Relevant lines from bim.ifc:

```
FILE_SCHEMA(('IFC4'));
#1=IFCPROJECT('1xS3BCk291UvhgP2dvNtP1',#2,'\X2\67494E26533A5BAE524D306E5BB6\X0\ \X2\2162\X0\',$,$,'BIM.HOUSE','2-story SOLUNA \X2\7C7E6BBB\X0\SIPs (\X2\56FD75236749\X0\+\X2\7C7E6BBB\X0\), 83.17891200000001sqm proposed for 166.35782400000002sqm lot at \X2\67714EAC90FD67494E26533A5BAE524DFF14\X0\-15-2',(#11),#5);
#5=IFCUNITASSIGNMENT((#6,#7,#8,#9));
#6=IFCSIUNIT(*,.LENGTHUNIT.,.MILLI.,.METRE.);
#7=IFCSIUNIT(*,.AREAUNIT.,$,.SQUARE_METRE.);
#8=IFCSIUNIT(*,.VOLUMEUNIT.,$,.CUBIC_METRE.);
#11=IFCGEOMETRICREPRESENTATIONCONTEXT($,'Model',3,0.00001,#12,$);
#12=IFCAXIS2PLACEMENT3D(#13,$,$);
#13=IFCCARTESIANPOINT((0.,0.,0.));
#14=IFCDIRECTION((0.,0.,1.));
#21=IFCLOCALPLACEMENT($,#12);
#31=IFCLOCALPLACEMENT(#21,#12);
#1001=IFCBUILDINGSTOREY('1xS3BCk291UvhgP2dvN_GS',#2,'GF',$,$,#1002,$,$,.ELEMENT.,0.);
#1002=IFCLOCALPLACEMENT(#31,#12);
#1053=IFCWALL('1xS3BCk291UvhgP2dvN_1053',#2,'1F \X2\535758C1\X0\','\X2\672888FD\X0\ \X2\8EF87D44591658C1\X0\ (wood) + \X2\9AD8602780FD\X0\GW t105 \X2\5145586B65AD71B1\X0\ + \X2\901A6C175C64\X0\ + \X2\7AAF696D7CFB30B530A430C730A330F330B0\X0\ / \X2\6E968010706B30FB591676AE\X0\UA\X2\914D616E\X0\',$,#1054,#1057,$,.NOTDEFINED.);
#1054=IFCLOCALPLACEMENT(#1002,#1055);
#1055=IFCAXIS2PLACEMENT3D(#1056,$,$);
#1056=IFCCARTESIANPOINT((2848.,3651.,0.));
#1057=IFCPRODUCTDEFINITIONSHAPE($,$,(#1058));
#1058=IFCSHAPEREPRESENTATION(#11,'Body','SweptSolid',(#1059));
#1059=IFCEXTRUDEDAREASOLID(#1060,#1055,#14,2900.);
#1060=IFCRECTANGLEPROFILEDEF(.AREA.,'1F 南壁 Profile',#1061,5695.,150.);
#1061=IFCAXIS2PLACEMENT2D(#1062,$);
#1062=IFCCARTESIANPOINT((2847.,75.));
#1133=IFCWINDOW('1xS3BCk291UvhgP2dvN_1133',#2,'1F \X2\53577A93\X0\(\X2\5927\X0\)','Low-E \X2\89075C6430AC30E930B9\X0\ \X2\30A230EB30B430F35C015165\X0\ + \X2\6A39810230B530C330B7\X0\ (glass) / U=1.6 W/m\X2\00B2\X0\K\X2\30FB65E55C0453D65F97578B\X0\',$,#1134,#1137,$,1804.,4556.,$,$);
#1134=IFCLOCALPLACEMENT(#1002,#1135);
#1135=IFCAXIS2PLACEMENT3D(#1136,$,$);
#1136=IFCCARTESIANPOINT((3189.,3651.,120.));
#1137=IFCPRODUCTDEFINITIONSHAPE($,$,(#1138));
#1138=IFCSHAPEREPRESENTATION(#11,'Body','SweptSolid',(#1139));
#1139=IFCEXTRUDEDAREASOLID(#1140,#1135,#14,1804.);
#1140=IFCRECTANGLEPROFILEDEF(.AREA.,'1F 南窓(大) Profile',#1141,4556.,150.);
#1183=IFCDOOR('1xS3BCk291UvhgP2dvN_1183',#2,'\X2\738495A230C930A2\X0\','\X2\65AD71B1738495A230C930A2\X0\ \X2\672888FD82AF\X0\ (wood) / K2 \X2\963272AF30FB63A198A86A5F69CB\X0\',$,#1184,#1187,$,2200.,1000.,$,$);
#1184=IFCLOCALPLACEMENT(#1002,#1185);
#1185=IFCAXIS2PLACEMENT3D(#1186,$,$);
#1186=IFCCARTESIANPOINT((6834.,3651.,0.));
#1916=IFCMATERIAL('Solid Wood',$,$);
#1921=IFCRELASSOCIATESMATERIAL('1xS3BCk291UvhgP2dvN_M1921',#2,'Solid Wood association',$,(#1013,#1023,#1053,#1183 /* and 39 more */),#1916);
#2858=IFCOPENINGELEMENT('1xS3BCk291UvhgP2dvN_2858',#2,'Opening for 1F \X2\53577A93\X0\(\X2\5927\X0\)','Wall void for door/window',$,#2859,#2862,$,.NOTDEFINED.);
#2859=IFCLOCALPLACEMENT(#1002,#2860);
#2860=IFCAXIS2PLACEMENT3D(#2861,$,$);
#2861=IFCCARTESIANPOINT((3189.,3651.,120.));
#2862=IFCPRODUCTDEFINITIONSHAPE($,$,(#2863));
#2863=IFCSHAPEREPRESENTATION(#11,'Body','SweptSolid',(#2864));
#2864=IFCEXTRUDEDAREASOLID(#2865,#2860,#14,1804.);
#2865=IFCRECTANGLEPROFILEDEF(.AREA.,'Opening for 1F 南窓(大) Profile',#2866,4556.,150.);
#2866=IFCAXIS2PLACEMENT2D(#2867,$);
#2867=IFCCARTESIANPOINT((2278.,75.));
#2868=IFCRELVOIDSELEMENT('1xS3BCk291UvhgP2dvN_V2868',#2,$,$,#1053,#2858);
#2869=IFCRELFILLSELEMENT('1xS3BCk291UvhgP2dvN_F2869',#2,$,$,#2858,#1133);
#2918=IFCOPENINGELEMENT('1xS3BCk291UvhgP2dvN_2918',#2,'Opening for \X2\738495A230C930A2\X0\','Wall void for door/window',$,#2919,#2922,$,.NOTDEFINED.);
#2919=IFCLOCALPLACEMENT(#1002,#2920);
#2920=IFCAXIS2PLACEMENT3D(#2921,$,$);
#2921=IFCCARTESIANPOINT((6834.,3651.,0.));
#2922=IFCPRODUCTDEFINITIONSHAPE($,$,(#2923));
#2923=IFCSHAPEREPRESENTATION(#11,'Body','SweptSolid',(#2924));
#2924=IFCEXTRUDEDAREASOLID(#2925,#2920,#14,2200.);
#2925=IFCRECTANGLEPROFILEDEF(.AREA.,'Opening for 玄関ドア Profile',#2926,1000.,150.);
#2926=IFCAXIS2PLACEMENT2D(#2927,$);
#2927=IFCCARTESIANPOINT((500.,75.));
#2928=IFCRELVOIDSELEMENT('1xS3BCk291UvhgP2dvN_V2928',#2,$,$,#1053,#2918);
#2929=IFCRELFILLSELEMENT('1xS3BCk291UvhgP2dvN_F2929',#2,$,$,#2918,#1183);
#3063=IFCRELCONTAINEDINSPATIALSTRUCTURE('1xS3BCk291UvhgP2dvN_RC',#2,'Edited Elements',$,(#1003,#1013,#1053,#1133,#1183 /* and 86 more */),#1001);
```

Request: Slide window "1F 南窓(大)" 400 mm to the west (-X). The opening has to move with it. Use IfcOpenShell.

```python
import ifcopenshell
import ifcopenshell.api.geometry
import ifcopenshell.util.placement
import ifcopenshell.util.unit

model = ifcopenshell.open("bim.ifc")
unit_scale = ifcopenshell.util.unit.calculate_unit_scale(model)

window = model.by_guid("1xS3BCk291UvhgP2dvN_1133")
opening = window.FillsVoids[0].RelatingOpeningElement
wall = opening.VoidsElements[0].RelatingBuildingElement

wall_matrix = ifcopenshell.util.placement.get_local_placement(wall.ObjectPlacement)
shift = wall_matrix[:3, 0] * -0.4 / unit_scale
before = ifcopenshell.util.placement.get_local_placement(window.ObjectPlacement)[:3, 3].copy()

# The window is not placed relative to its opening, so move both.
for product in (opening, window):
    matrix = ifcopenshell.util.placement.get_local_placement(product.ObjectPlacement)
    matrix[:3, 3] += shift
    ifcopenshell.api.geometry.edit_object_placement(model, product=product, matrix=matrix, is_si=False)

after = ifcopenshell.util.placement.get_local_placement(window.ObjectPlacement)[:3, 3]
print("window moved by", (after - before).round(3) + 0.0)

model.write("bim_edited.ifc")
```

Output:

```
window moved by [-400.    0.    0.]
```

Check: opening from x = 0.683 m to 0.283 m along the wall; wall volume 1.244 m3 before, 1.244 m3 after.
